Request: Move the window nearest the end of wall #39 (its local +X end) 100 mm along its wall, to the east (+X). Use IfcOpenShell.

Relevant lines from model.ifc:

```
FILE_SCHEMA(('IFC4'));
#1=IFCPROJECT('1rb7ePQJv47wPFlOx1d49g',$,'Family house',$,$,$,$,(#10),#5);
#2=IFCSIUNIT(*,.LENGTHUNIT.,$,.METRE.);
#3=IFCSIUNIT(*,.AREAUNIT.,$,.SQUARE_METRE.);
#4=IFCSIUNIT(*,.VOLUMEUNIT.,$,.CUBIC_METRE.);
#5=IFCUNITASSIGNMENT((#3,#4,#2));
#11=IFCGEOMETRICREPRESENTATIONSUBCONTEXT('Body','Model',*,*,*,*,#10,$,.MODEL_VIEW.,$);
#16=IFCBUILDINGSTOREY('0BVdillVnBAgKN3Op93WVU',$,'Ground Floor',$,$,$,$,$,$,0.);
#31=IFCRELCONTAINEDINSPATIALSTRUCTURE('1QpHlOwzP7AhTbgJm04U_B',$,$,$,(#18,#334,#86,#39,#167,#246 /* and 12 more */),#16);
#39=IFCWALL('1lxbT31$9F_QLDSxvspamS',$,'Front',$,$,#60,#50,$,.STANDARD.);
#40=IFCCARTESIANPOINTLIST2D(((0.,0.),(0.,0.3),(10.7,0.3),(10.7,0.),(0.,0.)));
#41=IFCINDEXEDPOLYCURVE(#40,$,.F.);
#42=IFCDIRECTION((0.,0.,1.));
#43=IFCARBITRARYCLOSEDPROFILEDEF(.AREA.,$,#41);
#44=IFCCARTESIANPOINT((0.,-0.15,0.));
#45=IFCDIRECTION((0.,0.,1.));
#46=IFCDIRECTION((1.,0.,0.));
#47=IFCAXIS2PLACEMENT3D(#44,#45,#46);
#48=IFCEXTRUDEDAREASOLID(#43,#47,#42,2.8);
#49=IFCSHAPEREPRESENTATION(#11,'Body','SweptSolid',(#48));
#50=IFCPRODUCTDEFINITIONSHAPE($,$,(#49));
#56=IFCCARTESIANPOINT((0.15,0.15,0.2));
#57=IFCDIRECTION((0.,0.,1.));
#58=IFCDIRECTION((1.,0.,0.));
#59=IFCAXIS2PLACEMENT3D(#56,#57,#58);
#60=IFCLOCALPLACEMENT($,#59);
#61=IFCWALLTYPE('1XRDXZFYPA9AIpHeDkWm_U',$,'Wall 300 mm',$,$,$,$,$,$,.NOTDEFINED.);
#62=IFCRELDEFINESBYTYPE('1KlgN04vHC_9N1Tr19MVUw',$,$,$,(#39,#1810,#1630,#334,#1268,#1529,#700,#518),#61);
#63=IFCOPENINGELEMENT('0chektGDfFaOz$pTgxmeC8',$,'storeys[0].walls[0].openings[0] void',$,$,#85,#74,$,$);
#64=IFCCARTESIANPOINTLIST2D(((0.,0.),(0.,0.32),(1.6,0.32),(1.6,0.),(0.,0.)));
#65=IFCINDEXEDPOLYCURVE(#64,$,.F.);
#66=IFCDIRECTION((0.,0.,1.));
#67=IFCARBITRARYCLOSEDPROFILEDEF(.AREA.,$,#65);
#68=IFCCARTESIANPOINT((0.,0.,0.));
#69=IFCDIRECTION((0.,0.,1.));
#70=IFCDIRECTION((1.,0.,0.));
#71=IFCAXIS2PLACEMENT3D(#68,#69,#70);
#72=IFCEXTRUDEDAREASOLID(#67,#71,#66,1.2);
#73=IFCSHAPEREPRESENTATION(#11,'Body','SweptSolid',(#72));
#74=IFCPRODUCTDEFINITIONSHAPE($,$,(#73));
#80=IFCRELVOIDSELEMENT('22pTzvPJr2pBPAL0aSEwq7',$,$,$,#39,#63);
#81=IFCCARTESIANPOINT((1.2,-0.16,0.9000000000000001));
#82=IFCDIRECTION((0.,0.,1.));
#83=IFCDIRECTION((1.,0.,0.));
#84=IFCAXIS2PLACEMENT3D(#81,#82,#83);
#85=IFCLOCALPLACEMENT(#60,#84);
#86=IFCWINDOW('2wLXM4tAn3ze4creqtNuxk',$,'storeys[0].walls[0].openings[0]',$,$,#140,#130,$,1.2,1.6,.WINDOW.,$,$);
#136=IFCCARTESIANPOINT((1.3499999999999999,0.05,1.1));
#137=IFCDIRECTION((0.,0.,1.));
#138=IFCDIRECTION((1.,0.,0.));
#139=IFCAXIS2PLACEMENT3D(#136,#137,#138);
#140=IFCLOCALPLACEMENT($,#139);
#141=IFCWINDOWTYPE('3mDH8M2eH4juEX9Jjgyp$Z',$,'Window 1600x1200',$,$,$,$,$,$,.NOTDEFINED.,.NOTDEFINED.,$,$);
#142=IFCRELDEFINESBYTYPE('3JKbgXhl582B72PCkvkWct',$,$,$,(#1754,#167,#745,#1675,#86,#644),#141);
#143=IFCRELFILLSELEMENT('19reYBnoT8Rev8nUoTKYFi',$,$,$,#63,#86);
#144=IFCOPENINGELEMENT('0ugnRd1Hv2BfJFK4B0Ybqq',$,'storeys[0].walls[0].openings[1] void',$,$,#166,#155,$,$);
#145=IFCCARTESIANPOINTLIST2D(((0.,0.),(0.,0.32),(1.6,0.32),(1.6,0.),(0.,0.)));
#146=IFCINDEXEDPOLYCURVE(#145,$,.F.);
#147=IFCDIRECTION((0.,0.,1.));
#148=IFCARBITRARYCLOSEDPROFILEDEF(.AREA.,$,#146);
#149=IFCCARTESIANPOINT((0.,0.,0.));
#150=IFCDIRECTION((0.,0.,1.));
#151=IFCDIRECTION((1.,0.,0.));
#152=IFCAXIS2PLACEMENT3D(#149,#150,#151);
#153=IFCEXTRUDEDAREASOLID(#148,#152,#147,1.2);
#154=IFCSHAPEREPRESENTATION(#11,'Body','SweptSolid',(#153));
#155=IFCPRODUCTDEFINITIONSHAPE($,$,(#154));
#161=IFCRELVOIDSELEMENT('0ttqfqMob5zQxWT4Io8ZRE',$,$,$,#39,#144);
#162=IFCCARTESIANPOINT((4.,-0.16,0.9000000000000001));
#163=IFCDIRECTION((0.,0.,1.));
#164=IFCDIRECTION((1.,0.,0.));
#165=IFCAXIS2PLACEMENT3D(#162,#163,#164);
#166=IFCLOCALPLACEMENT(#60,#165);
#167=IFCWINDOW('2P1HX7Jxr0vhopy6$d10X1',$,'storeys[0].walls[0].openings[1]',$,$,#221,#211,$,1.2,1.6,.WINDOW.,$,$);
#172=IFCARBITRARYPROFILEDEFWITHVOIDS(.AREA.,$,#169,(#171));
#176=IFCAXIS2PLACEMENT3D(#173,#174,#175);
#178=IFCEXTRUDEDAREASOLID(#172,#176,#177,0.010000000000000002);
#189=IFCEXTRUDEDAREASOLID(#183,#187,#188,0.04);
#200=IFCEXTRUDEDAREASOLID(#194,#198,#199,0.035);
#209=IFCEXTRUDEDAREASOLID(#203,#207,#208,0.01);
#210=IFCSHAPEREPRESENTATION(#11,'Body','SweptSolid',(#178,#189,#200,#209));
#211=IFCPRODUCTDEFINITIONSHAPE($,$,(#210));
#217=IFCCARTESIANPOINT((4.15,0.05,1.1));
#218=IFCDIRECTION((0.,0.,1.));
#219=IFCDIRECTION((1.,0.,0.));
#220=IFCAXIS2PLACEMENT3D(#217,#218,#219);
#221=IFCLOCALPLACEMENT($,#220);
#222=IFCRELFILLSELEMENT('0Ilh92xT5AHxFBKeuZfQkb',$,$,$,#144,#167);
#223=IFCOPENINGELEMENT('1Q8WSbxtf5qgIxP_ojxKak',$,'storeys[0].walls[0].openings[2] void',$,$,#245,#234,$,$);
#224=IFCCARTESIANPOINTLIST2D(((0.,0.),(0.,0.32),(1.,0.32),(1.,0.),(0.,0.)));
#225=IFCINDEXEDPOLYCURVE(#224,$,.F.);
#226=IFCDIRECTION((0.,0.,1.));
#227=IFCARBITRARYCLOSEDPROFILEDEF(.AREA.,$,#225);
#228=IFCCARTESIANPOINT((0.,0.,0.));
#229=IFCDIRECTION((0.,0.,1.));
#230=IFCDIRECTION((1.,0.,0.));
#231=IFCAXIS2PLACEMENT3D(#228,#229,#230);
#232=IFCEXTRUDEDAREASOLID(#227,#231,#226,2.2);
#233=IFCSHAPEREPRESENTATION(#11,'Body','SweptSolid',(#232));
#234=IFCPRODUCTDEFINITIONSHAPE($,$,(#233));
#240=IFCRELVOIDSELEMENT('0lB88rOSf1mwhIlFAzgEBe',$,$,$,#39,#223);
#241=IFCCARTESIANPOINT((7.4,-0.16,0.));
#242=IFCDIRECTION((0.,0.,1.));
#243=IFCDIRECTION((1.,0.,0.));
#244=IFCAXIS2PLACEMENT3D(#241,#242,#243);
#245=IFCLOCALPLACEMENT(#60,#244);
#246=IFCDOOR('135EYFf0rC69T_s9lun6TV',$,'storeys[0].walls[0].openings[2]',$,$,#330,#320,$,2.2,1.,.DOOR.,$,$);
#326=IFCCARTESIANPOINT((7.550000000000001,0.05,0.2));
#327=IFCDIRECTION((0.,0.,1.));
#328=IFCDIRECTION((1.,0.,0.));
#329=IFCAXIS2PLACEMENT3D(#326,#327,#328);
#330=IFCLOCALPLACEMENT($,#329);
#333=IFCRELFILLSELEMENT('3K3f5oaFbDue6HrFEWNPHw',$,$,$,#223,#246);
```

```python
import ifcopenshell
import ifcopenshell.api.geometry
import ifcopenshell.util.placement

model = ifcopenshell.open("model.ifc")

window = model.by_guid("2P1HX7Jxr0vhopy6$d10X1")
opening = window.FillsVoids[0].RelatingOpeningElement
wall = opening.VoidsElements[0].RelatingBuildingElement

wall_matrix = ifcopenshell.util.placement.get_local_placement(wall.ObjectPlacement)
shift = wall_matrix[:3, 0] * 0.1
before = ifcopenshell.util.placement.get_local_placement(window.ObjectPlacement)[:3, 3].copy()

# The window is not placed relative to its opening, so move both.
for product in (opening, window):
    matrix = ifcopenshell.util.placement.get_local_placement(product.ObjectPlacement)
    matrix[:3, 3] += shift
    ifcopenshell.api.geometry.edit_object_placement(model, product=product, matrix=matrix, is_si=False)

after = ifcopenshell.util.placement.get_local_placement(window.ObjectPlacement)[:3, 3]
print("window moved by", (after - before).round(3) + 0.0)

model.write("model_edited.ifc")
```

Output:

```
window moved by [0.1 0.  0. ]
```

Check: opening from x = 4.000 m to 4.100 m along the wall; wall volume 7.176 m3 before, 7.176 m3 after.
